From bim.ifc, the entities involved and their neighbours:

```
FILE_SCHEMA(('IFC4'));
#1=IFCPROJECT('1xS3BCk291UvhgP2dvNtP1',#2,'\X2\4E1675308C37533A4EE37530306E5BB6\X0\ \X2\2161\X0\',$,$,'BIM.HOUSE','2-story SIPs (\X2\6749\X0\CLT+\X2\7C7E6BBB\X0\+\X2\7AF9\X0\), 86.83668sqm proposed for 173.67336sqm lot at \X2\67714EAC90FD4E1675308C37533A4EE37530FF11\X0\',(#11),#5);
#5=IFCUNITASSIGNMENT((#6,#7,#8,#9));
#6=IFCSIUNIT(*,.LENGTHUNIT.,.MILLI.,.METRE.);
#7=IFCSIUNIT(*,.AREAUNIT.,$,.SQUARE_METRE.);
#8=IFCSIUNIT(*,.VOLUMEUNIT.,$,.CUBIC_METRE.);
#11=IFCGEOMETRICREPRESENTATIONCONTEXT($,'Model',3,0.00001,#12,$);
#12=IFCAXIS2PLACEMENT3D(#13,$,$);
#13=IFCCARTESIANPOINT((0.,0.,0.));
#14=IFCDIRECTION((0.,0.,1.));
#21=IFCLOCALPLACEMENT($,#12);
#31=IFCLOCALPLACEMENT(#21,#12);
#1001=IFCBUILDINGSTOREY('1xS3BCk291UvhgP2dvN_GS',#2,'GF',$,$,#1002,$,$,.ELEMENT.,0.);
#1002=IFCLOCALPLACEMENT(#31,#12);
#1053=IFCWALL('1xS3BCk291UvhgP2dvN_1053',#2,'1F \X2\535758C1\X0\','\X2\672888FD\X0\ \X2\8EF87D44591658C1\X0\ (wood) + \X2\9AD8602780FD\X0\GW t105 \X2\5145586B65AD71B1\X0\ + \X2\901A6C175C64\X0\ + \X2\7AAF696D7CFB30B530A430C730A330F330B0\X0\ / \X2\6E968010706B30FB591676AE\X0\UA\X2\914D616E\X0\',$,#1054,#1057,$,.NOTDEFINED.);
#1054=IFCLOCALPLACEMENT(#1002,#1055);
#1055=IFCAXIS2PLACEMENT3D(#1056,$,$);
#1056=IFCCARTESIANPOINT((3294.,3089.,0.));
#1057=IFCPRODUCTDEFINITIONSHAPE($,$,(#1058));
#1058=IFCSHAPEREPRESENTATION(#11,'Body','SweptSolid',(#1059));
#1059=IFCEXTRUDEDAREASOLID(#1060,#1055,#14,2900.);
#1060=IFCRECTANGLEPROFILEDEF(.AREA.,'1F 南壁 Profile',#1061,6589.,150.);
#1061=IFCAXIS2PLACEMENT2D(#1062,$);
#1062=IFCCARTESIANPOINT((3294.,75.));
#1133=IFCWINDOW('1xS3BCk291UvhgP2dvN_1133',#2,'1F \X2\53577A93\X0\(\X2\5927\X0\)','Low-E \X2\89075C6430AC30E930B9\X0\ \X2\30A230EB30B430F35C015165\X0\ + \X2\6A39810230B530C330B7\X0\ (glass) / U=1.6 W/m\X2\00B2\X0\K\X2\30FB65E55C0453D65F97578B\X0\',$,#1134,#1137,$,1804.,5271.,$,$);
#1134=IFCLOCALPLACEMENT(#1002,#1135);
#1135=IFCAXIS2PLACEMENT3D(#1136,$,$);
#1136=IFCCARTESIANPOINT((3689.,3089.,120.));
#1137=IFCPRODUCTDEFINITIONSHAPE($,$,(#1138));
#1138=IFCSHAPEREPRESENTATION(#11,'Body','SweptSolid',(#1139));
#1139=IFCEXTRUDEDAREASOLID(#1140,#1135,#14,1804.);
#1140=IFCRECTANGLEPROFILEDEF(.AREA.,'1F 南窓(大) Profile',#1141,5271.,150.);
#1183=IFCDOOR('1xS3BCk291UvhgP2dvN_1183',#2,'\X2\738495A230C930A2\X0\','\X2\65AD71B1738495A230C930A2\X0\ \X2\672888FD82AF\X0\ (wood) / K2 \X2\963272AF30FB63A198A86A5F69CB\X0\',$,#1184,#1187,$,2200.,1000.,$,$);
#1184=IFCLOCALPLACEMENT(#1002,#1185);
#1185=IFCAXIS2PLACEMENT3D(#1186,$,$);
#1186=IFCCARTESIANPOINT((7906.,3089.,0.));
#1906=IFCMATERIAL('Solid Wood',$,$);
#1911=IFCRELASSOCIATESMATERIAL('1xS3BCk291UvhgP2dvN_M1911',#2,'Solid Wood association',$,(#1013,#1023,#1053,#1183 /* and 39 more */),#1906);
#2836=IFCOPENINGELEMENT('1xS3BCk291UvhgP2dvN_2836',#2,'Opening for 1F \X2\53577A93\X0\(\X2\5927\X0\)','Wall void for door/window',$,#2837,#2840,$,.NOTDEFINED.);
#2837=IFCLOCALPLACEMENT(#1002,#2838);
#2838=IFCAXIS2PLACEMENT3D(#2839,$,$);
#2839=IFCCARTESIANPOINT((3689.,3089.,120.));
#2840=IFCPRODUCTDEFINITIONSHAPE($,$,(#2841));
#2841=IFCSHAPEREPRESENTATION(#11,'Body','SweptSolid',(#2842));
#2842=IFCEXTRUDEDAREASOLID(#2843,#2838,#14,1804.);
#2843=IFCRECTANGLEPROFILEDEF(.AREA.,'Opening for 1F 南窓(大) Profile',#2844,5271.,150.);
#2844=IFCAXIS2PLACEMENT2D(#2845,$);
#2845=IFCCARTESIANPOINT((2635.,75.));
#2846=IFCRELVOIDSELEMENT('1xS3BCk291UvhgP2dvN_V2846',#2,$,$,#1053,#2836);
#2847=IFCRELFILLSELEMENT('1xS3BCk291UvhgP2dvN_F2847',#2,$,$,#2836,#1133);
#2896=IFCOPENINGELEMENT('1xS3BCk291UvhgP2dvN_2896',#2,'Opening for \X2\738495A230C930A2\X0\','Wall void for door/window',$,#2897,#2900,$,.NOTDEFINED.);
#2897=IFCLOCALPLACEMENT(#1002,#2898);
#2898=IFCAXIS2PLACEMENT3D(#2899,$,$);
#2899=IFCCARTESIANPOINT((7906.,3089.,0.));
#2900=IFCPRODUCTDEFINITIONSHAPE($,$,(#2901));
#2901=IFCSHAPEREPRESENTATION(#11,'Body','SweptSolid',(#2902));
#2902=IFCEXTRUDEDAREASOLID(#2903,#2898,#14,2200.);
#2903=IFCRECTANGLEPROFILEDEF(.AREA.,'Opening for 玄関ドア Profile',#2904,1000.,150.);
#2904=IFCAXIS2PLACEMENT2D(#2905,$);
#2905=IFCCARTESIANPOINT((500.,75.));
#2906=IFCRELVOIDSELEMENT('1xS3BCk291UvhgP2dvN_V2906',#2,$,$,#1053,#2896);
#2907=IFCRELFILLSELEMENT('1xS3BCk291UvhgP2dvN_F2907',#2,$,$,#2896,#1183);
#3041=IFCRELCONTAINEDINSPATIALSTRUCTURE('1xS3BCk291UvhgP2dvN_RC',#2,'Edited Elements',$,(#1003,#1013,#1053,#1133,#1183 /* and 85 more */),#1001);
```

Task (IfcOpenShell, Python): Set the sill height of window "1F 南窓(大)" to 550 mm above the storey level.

```python
import numpy as np
import ifcopenshell
import ifcopenshell.api.geometry
import ifcopenshell.geom
import ifcopenshell.util.element
import ifcopenshell.util.placement
import ifcopenshell.util.shape
import ifcopenshell.util.unit

model = ifcopenshell.open("bim.ifc")
unit_scale = ifcopenshell.util.unit.calculate_unit_scale(model)

window = model.by_id(1133)
opening = window.FillsVoids[0].RelatingOpeningElement
storey = ifcopenshell.util.element.get_container(window, ifc_class="IfcBuildingStorey")
level = ifcopenshell.util.placement.get_local_placement(storey.ObjectPlacement)[2, 3]

# The opening's origin need not be at the sill, so measure its lowest point.
shape = ifcopenshell.geom.create_shape(ifcopenshell.geom.settings(), opening)
bottom = ifcopenshell.util.shape.get_shape_bottom_elevation(shape, shape.geometry) / unit_scale
dz = level + 0.55 / unit_scale - bottom

shift = np.array([0.0, 0.0, dz])
# The window is not placed relative to its opening, so move both.
for product in (opening, window):
    matrix = ifcopenshell.util.placement.get_local_placement(product.ObjectPlacement)
    matrix[:3, 3] += shift
    ifcopenshell.api.geometry.edit_object_placement(model, product=product, matrix=matrix, is_si=False)

print(f"moved by {dz * unit_scale:+.3f} m")

model.write("bim_rev.ifc")
```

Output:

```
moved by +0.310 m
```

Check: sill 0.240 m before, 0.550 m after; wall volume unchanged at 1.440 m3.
